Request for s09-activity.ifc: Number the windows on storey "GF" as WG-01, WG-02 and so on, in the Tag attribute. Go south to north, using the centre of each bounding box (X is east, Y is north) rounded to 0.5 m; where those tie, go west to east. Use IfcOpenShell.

First a look at what the model holds.

```python
import ifcopenshell
import ifcopenshell.util.element
import ifcopenshell.util.placement

model = ifcopenshell.open("s09-activity.ifc")
print(model.schema)
storey = next(s for s in model.by_type("IfcBuildingStorey") if s.Name == "GF")
windows = [e for e in ifcopenshell.util.element.get_decomposition(storey) if e.is_a("IfcWindow")]
for e in sorted(windows, key=lambda e: e.id()):
    origin = ifcopenshell.util.placement.get_local_placement(e.ObjectPlacement)[:3, 3]
    print(e.id(), e.Tag, e.Name, origin.round(2) + 0.0, sep=" | ")
```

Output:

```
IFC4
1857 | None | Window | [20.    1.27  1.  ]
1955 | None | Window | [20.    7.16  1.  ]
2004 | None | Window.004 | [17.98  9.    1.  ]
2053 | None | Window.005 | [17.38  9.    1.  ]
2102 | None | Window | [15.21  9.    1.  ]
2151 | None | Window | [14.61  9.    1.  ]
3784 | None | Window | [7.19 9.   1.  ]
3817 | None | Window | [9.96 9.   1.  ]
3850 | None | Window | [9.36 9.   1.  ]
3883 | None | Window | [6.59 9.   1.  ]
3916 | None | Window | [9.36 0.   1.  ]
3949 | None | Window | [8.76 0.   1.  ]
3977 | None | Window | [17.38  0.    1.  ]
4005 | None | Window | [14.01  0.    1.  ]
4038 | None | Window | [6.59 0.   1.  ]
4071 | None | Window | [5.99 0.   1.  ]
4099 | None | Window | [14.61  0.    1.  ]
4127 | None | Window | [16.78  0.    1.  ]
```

```python
import ifcopenshell
import ifcopenshell.geom
import ifcopenshell.util.element
import ifcopenshell.util.shape

model = ifcopenshell.open("s09-activity.ifc")
settings = ifcopenshell.geom.settings()
settings.set("use-world-coords", True)


def centre(element):
    shape = ifcopenshell.geom.create_shape(settings, element)
    return ifcopenshell.util.shape.get_bbox_centroid(shape.geometry)


storey = next(s for s in model.by_type("IfcBuildingStorey") if s.Name == "GF")
windows = [e for e in ifcopenshell.util.element.get_decomposition(storey) if e.is_a("IfcWindow")]

# Insertion points can sit at a corner or the storey origin, so sort by the geometry (in metres).
centres = {e: centre(e) for e in windows}
windows.sort(key=lambda e: (round(centres[e][1] / 0.5), centres[e][0]))

for i, e in enumerate(windows, start=1):
    number = f"WG-{i:02d}"
    e.Tag = number
    print(e.id(), number)

model.write("s09-activity_updated.ifc")
```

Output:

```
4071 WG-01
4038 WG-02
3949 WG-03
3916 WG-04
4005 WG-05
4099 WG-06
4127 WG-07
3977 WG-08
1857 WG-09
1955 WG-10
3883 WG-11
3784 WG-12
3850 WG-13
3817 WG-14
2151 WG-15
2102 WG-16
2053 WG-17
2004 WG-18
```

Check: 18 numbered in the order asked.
